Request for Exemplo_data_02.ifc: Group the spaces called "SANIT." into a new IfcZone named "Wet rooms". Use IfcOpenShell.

First a look at what the model holds.

```python
import ifcopenshell

model = ifcopenshell.open("Exemplo_data_02.ifc")
print(model.schema)
seen = {}
for space in model.by_type("IfcSpace"):
    seen[space.LongName] = seen.get(space.LongName, 0) + 1
for name, count in sorted(seen.items(), key=str):
    print(count, "x", name)
print("zones:", [z.Name for z in model.by_type("IfcZone")][:20])
```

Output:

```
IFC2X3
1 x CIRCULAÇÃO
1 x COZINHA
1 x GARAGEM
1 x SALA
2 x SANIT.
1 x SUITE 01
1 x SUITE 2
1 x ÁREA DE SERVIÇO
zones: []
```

```python
import ifcopenshell
import ifcopenshell.api.group
import ifcopenshell.api.root

model = ifcopenshell.open("Exemplo_data_02.ifc")

names = {"SANIT."}
spaces = [s for s in model.by_type("IfcSpace") if s.LongName in names]

zone = ifcopenshell.api.root.create_entity(model, ifc_class="IfcZone", name="Wet rooms")
ifcopenshell.api.group.assign_group(model, products=spaces, group=zone)
print(len(spaces), "spaces in", zone.Name)

model.write("Exemplo_data_02-out.ifc")
```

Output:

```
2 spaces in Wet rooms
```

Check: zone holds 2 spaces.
